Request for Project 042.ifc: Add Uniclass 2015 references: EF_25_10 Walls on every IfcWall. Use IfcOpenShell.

First a look at what the model holds.

```python
import ifcopenshell

model = ifcopenshell.open("Project 042.ifc")
print(model.schema)
print("classifications:", [c.Name for c in model.by_type("IfcClassification")])
for ifc_class in ("IfcDoor", "IfcRoof", "IfcStair", "IfcWall", "IfcWindow"):
    print(ifc_class, len(model.by_type(ifc_class)))
```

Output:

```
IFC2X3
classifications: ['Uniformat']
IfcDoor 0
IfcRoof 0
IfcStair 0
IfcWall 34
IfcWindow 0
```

```python
import ifcopenshell
import ifcopenshell.api.classification

model = ifcopenshell.open("Project 042.ifc")

# IFC2X3 requires Source and Edition and has no link from the project to the system.
system = model.create_entity("IfcClassification", Source="NBS", Edition="2015", Name="Uniclass 2015")

codes = {
    "IfcWall": ("EF_25_10", "Walls"),
}
for ifc_class, (code, name) in codes.items():
    products = model.by_type(ifc_class)
    ifcopenshell.api.classification.add_reference(
        model, products=products, classification=system, identification=code, name=name
    )
    print(code, len(products))

model.write("Project 042_rev.ifc")
```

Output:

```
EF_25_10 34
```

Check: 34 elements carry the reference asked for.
